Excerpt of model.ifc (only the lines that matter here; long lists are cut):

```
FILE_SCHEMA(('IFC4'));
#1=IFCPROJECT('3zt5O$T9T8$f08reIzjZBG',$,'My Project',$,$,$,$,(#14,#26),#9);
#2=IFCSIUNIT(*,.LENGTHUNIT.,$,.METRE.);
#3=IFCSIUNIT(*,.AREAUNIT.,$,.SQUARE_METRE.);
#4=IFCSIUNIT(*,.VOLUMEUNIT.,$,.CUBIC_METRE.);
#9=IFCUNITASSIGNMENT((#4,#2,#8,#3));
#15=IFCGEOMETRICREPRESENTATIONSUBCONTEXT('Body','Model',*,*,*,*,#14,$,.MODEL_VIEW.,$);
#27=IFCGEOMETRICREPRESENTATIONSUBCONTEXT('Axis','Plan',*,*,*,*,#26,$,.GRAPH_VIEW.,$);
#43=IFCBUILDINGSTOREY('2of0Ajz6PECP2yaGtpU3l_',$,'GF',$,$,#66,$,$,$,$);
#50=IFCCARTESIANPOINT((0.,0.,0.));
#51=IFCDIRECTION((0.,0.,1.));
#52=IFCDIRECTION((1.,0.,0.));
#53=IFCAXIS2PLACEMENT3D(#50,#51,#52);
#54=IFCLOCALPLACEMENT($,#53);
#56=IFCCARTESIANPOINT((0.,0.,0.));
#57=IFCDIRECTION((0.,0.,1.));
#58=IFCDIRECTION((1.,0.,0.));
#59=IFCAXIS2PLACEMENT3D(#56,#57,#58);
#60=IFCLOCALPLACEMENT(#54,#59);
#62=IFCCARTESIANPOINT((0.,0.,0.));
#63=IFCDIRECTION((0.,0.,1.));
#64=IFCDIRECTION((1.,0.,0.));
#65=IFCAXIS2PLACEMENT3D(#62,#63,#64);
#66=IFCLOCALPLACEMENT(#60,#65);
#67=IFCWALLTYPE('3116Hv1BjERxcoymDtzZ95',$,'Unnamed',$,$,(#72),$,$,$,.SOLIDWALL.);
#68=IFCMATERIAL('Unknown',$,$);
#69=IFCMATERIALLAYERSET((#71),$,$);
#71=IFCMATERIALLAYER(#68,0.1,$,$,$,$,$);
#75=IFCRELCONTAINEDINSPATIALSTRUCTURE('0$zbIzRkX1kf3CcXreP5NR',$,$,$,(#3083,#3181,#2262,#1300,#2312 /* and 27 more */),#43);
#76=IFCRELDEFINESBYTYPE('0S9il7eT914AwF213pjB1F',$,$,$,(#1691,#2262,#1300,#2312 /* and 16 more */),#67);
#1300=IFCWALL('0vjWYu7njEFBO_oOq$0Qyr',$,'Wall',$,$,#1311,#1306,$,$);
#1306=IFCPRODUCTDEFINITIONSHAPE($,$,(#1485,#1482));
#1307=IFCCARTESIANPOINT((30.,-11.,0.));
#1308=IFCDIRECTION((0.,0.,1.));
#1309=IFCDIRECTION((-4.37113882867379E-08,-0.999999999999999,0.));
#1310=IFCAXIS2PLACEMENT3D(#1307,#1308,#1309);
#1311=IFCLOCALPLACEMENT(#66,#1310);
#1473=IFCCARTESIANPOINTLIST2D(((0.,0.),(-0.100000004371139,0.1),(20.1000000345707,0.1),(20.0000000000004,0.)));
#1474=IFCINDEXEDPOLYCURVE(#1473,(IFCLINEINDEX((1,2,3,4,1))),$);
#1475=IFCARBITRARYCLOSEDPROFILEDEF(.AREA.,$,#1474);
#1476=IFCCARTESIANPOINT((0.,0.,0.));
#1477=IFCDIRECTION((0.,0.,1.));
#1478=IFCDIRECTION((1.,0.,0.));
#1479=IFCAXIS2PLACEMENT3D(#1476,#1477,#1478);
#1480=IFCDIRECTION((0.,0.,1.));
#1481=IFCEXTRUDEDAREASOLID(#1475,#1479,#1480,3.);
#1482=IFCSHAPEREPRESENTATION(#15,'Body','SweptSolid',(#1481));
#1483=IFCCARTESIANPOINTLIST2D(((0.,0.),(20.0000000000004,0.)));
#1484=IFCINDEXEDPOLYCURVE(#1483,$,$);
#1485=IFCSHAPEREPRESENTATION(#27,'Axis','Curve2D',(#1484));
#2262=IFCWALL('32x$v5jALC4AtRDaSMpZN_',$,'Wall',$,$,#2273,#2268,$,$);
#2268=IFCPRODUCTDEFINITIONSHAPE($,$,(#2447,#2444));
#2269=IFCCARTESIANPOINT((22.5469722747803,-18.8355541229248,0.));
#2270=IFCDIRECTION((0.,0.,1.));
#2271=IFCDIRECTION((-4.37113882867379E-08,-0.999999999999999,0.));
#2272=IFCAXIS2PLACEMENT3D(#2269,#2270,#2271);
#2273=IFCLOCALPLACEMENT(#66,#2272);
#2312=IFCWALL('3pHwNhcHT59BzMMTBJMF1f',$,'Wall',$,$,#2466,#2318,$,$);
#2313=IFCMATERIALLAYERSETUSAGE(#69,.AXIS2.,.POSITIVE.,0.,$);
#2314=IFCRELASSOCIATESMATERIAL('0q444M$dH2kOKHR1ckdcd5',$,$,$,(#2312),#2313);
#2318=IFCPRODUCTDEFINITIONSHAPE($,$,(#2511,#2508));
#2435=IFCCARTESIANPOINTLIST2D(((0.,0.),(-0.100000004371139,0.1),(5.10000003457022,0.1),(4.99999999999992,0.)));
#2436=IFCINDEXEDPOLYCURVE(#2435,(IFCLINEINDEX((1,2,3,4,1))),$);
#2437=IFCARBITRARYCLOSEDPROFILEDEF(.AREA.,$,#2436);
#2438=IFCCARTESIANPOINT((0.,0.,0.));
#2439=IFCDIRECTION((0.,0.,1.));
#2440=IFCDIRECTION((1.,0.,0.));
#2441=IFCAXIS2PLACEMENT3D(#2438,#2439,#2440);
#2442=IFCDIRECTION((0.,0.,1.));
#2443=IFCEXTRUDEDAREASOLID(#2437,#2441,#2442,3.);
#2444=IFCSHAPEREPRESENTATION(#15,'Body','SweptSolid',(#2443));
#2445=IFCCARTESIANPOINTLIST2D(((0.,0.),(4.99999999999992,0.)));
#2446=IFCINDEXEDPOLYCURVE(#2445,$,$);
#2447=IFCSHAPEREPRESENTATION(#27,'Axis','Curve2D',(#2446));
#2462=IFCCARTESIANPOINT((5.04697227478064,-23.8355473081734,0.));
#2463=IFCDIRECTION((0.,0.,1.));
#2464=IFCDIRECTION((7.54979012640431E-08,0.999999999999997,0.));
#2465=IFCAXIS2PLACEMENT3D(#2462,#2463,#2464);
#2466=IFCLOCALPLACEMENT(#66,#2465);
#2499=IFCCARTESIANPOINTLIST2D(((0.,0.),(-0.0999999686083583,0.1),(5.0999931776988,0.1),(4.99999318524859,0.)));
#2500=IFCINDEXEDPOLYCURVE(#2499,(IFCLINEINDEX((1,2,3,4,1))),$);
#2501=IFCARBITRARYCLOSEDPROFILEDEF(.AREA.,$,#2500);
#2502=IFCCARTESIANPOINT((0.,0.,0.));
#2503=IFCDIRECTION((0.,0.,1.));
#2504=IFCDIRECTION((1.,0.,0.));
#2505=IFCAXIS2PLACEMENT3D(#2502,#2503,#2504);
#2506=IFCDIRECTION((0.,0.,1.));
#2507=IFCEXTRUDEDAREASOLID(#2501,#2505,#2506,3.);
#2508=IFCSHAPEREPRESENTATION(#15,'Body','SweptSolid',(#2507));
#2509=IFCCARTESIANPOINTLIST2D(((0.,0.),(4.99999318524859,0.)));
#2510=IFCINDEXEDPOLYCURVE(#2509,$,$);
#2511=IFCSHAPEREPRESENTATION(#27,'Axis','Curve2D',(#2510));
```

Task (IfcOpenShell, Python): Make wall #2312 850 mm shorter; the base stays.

```python
import ifcopenshell
import ifcopenshell.geom
import ifcopenshell.util.representation
import ifcopenshell.util.shape
import ifcopenshell.util.unit

model = ifcopenshell.open("model.ifc")
unit_scale = ifcopenshell.util.unit.calculate_unit_scale(model)
settings = ifcopenshell.geom.settings()


def volume(element):
    """Net volume in cubic metres, openings subtracted."""
    shape = ifcopenshell.geom.create_shape(settings, element)
    return ifcopenshell.util.shape.get_volume(shape.geometry)


wall = model.by_id(2312)
before = volume(wall)

body = ifcopenshell.util.representation.get_representation(wall, "Model", "Body")
solid = body.Items[0]
old_height = solid.Depth
solid.Depth -= 0.85 / unit_scale
after = volume(wall)

print(f"height {old_height:g} -> {solid.Depth:g}, volume {before:.3f} -> {after:.3f} m3")

model.write("model-out.ifc")
```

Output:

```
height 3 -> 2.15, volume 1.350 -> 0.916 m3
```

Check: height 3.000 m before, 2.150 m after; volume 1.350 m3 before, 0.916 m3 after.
